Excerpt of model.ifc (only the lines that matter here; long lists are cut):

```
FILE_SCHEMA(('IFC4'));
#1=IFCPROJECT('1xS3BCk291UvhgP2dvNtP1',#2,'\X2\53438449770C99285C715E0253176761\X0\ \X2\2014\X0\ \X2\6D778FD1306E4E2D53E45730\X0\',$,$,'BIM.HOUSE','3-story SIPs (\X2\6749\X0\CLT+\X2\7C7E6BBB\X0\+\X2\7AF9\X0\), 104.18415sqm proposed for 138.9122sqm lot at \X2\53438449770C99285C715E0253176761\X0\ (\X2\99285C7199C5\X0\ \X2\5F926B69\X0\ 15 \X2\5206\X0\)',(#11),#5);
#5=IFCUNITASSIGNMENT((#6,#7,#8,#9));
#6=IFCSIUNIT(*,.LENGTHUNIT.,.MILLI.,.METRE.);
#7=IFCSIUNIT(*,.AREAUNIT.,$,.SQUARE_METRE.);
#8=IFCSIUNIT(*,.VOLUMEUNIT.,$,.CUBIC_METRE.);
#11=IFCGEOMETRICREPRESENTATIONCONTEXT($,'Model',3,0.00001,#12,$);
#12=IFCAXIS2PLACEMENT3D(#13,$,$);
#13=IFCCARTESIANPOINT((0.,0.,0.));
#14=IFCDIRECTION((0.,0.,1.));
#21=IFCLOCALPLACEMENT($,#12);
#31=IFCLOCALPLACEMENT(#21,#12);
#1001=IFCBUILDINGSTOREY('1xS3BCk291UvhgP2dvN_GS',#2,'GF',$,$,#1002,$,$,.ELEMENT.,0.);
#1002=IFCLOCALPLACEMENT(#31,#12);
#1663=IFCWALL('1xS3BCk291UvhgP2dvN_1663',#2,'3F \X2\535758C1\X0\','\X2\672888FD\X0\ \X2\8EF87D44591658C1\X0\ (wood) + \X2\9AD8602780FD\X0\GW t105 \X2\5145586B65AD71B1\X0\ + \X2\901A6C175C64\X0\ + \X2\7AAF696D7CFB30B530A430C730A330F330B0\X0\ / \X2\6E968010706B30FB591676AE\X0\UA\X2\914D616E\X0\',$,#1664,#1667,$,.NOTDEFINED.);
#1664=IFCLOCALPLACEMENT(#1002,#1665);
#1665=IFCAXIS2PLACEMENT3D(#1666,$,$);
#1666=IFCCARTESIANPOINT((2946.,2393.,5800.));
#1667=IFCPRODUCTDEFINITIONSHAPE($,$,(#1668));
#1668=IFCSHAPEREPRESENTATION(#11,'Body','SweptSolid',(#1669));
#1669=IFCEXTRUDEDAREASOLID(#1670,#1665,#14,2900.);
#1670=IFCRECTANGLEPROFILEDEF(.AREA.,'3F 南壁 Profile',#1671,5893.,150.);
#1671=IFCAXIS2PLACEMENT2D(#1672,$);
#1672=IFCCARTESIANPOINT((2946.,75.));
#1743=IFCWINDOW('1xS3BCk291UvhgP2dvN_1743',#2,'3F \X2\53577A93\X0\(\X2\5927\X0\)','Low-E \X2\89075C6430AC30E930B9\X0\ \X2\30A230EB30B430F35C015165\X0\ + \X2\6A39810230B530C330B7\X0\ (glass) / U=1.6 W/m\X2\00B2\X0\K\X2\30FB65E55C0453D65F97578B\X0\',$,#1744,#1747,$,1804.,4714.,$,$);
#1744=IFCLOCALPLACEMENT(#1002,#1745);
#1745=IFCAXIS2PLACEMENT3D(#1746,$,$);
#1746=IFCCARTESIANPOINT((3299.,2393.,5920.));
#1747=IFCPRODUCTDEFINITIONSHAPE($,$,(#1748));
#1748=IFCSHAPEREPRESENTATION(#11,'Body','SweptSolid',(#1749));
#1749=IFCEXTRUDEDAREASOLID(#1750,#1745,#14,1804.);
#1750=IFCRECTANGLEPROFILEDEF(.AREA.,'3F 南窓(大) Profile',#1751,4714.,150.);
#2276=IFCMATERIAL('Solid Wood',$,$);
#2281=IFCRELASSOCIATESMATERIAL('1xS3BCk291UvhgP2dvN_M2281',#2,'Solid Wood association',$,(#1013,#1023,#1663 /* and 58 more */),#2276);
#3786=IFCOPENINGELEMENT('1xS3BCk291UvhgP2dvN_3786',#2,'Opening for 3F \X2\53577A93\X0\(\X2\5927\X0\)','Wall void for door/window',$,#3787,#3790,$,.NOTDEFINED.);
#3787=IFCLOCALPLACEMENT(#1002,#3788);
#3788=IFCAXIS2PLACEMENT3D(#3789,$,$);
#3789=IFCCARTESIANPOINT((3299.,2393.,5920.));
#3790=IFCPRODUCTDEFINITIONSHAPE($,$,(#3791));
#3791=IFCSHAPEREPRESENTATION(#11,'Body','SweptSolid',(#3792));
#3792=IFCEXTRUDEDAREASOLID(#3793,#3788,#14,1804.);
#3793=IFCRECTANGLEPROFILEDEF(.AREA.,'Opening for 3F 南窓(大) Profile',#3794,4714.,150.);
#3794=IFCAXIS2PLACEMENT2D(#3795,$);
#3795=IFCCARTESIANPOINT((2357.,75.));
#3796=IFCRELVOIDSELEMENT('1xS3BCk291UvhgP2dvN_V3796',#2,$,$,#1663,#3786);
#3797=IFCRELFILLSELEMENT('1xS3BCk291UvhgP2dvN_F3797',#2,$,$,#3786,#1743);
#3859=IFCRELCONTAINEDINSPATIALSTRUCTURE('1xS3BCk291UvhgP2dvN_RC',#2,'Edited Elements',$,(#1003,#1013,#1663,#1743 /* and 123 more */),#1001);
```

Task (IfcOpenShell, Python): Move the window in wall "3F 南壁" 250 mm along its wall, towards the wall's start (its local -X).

```python
import ifcopenshell
import ifcopenshell.api.geometry
import ifcopenshell.util.placement
import ifcopenshell.util.unit

model = ifcopenshell.open("model.ifc")
unit_scale = ifcopenshell.util.unit.calculate_unit_scale(model)

window = model.by_guid("1xS3BCk291UvhgP2dvN_1743")
opening = window.FillsVoids[0].RelatingOpeningElement
wall = opening.VoidsElements[0].RelatingBuildingElement

wall_matrix = ifcopenshell.util.placement.get_local_placement(wall.ObjectPlacement)
shift = wall_matrix[:3, 0] * -0.25 / unit_scale
before = ifcopenshell.util.placement.get_local_placement(window.ObjectPlacement)[:3, 3].copy()

# The window is not placed relative to its opening, so move both.
for product in (opening, window):
    matrix = ifcopenshell.util.placement.get_local_placement(product.ObjectPlacement)
    matrix[:3, 3] += shift
    ifcopenshell.api.geometry.edit_object_placement(model, product=product, matrix=matrix, is_si=False)

after = ifcopenshell.util.placement.get_local_placement(window.ObjectPlacement)[:3, 3]
print("window moved by", (after - before).round(3) + 0.0)

model.write("model_rev.ifc")
```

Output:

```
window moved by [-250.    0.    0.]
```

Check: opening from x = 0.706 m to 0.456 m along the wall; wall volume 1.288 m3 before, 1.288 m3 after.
